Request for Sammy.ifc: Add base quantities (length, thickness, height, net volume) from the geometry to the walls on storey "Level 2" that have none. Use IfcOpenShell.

First a look at what the model holds.

```python
import ifcopenshell
import ifcopenshell.util.element
import ifcopenshell.util.unit

model = ifcopenshell.open("Sammy.ifc")
print(model.schema)
for unit_type in ("LENGTHUNIT", "AREAUNIT", "VOLUMEUNIT"):
    print(unit_type, ifcopenshell.util.unit.calculate_unit_scale(model, unit_type))
storey = next(s for s in model.by_type("IfcBuildingStorey") if s.Name == "Level 2")
walls = [e for e in ifcopenshell.util.element.get_decomposition(storey) if e.is_a("IfcWall")]
for e in sorted(walls, key=lambda e: e.id()):
    print(e.id(), e.is_a(), e.Name, list(ifcopenshell.util.element.get_psets(e, qtos_only=True)), sep=" | ")
```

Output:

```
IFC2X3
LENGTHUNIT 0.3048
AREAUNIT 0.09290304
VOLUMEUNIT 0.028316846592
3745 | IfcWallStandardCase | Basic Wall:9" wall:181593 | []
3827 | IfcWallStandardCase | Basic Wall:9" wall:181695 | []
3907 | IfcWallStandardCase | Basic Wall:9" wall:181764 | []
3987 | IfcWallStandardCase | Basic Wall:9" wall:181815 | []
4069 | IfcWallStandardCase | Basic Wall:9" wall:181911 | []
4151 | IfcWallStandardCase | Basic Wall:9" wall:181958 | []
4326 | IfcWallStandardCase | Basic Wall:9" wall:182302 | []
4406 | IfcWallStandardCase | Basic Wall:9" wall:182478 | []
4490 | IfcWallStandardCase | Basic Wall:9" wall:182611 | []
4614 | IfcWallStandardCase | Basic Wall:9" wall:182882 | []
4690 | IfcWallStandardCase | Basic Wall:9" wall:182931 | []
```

```python
import ifcopenshell
import ifcopenshell.api.pset
import ifcopenshell.geom
import ifcopenshell.util.element
import ifcopenshell.util.shape
import ifcopenshell.util.unit

model = ifcopenshell.open("Sammy.ifc")
unit_scale = ifcopenshell.util.unit.calculate_unit_scale(model)
volume_scale = ifcopenshell.util.unit.calculate_unit_scale(model, "VOLUMEUNIT")
settings = ifcopenshell.geom.settings()

storey = next(s for s in model.by_type("IfcBuildingStorey") if s.Name == "Level 2")
walls = [e for e in ifcopenshell.util.element.get_decomposition(storey) if e.is_a("IfcWall")]

for e in sorted(walls, key=lambda e: e.id()):
    if ifcopenshell.util.element.get_psets(e, qtos_only=True, should_inherit=False):
        continue
    # Geometry comes back in metres, in the element's own axes.
    shape = ifcopenshell.geom.create_shape(settings, e)
    values = {
        "Length": ifcopenshell.util.shape.get_x(shape.geometry) / unit_scale,
        "Width": ifcopenshell.util.shape.get_y(shape.geometry) / unit_scale,
        "Height": ifcopenshell.util.shape.get_z(shape.geometry) / unit_scale,
        "NetVolume": ifcopenshell.util.shape.get_volume(shape.geometry) / volume_scale,
    }
    qto = ifcopenshell.api.pset.add_qto(model, product=e, name="BaseQuantities")
    ifcopenshell.api.pset.edit_qto(model, qto=qto, properties=values)
    print(e.id(), {k: round(v, 3) for k, v in values.items()})

model.write("Sammy_edited.ifc")
```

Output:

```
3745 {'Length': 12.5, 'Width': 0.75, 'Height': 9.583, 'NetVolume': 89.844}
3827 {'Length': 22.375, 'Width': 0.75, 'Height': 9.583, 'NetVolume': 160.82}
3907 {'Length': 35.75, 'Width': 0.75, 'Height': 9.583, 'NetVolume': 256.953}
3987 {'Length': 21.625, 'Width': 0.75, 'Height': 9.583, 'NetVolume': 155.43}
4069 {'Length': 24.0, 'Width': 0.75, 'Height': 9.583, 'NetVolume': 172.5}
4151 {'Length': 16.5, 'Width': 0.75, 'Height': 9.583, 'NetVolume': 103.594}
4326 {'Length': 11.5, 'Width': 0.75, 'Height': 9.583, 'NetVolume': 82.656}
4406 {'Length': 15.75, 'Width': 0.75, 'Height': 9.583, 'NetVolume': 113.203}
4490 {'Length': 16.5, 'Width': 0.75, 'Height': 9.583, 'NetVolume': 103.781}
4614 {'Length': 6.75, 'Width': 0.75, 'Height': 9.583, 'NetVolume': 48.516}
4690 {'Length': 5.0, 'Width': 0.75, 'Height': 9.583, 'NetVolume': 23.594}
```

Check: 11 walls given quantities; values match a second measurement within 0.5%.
